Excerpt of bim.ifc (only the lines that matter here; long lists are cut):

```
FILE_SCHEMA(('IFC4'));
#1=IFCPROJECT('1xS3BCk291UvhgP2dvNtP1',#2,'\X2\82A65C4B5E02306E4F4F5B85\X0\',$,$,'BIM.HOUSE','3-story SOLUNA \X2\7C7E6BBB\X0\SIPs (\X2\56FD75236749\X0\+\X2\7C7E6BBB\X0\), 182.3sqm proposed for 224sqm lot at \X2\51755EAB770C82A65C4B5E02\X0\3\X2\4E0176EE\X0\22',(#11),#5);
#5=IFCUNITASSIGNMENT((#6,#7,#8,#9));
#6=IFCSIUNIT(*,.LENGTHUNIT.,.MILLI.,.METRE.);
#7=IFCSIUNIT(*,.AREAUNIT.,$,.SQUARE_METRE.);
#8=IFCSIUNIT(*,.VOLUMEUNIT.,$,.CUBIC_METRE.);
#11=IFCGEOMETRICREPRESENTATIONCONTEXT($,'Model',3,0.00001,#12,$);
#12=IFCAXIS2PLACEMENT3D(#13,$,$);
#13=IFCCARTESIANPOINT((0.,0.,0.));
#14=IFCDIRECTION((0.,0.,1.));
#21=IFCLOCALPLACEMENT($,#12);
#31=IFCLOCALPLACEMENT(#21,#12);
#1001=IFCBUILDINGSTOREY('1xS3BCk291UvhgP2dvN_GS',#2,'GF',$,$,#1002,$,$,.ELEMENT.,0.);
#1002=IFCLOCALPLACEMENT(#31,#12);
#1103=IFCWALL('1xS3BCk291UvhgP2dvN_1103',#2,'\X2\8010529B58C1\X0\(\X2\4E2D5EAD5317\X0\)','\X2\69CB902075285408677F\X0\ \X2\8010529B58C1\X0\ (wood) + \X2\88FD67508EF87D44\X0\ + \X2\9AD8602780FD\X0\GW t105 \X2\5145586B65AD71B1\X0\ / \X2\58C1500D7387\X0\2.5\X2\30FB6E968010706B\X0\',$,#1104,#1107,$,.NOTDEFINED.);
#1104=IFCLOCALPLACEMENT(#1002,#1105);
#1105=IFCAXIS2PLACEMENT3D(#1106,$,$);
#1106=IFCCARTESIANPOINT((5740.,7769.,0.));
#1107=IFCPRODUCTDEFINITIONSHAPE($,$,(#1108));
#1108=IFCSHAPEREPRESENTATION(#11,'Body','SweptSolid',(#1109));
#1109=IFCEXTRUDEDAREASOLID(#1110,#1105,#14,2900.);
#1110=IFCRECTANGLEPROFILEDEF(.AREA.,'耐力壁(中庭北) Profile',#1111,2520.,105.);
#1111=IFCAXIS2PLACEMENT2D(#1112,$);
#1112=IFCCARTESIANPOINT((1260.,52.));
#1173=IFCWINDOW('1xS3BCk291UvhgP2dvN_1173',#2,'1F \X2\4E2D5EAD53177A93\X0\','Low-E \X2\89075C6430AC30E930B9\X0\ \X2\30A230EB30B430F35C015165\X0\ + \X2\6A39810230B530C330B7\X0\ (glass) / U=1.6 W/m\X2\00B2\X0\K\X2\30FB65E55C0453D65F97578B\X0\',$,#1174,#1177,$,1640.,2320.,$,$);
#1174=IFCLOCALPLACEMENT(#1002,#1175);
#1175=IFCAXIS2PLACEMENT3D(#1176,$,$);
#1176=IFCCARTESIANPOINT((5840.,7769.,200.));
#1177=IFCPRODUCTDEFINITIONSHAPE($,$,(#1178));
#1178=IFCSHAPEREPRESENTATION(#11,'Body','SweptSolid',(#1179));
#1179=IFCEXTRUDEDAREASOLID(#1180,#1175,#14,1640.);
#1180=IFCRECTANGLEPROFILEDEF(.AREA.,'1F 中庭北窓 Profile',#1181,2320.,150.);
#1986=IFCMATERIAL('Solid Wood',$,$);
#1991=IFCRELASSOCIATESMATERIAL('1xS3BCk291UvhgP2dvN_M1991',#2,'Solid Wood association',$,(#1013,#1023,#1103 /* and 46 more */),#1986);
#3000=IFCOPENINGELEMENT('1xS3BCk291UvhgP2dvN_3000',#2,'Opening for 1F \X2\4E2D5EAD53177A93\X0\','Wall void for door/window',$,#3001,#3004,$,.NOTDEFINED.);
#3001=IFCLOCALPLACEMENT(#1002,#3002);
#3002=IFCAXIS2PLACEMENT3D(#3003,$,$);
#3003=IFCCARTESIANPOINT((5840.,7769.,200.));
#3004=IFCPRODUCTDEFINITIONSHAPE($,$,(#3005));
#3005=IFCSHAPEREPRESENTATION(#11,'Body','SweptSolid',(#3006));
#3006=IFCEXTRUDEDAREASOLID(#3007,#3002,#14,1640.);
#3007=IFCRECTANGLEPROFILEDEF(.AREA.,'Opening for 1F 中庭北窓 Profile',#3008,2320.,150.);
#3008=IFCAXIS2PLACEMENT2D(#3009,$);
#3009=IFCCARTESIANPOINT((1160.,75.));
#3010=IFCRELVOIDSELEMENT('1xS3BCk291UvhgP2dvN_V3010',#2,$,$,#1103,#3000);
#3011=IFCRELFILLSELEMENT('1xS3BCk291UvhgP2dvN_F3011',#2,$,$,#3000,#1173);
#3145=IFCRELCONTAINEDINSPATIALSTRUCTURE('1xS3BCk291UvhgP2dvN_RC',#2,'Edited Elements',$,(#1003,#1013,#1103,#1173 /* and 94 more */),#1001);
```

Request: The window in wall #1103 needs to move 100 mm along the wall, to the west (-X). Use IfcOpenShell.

```python
import ifcopenshell
import ifcopenshell.api.geometry
import ifcopenshell.util.placement

model = ifcopenshell.open("bim.ifc")

window = model.by_id(1173)
opening = window.FillsVoids[0].RelatingOpeningElement
wall = opening.VoidsElements[0].RelatingBuildingElement

wall_matrix = ifcopenshell.util.placement.get_local_placement(wall.ObjectPlacement)
shift = wall_matrix[:3, 0] * -100.0
before = ifcopenshell.util.placement.get_local_placement(window.ObjectPlacement)[:3, 3].copy()

# The window is not placed relative to its opening, so move both.
for product in (opening, window):
    matrix = ifcopenshell.util.placement.get_local_placement(product.ObjectPlacement)
    matrix[:3, 3] += shift
    ifcopenshell.api.geometry.edit_object_placement(model, product=product, matrix=matrix, is_si=False)

after = ifcopenshell.util.placement.get_local_placement(window.ObjectPlacement)[:3, 3]
print("window moved by", (after - before).round(3) + 0.0)

model.write("bim_v2.ifc")
```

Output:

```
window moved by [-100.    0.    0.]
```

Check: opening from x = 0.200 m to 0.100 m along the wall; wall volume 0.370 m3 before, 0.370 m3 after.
